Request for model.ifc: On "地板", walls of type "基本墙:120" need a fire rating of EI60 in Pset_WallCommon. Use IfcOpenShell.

First a look at what the model holds.

```python
import ifcopenshell
import ifcopenshell.util.element

model = ifcopenshell.open("model.ifc")
print(model.schema)
storey = next(s for s in model.by_type("IfcBuildingStorey") if s.Name == "地板")
walls = [e for e in ifcopenshell.util.element.get_decomposition(storey) if e.is_a("IfcWall")]
seen = {}
for e in walls:
    element_type = ifcopenshell.util.element.get_type(e)
    key = (element_type.Name if element_type != e and element_type else None, ifcopenshell.util.element.get_pset(e, "Pset_WallCommon", "FireRating"))
    seen[key] = seen.get(key, 0) + 1
for (name, value), count in sorted(seen.items(), key=str):
    print(count, "x", name, "|", value)
```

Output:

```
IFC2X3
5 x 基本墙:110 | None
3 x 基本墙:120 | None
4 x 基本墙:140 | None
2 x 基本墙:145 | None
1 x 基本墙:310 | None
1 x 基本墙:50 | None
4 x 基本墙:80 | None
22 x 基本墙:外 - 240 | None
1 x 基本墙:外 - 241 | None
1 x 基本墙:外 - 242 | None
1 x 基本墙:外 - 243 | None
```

```python
import ifcopenshell
import ifcopenshell.api.pset
import ifcopenshell.util.element

model = ifcopenshell.open("model.ifc")

storey = next(s for s in model.by_type("IfcBuildingStorey") if s.Name == "地板")
walls = [e for e in ifcopenshell.util.element.get_decomposition(storey) if e.is_a("IfcWall")]

count = 0
for e in walls:
    element_type = ifcopenshell.util.element.get_type(e)
    if element_type in (None, e) or element_type.Name != "基本墙:120":
        continue
    # add_pset returns the element's existing set when there is one.
    pset = ifcopenshell.api.pset.add_pset(model, product=e, name="Pset_WallCommon")
    ifcopenshell.api.pset.edit_pset(model, pset=pset, properties={"FireRating": "EI60"})
    count += 1

print(count, "walls updated")

model.write("model-out.ifc")
```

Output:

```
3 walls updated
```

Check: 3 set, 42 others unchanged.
